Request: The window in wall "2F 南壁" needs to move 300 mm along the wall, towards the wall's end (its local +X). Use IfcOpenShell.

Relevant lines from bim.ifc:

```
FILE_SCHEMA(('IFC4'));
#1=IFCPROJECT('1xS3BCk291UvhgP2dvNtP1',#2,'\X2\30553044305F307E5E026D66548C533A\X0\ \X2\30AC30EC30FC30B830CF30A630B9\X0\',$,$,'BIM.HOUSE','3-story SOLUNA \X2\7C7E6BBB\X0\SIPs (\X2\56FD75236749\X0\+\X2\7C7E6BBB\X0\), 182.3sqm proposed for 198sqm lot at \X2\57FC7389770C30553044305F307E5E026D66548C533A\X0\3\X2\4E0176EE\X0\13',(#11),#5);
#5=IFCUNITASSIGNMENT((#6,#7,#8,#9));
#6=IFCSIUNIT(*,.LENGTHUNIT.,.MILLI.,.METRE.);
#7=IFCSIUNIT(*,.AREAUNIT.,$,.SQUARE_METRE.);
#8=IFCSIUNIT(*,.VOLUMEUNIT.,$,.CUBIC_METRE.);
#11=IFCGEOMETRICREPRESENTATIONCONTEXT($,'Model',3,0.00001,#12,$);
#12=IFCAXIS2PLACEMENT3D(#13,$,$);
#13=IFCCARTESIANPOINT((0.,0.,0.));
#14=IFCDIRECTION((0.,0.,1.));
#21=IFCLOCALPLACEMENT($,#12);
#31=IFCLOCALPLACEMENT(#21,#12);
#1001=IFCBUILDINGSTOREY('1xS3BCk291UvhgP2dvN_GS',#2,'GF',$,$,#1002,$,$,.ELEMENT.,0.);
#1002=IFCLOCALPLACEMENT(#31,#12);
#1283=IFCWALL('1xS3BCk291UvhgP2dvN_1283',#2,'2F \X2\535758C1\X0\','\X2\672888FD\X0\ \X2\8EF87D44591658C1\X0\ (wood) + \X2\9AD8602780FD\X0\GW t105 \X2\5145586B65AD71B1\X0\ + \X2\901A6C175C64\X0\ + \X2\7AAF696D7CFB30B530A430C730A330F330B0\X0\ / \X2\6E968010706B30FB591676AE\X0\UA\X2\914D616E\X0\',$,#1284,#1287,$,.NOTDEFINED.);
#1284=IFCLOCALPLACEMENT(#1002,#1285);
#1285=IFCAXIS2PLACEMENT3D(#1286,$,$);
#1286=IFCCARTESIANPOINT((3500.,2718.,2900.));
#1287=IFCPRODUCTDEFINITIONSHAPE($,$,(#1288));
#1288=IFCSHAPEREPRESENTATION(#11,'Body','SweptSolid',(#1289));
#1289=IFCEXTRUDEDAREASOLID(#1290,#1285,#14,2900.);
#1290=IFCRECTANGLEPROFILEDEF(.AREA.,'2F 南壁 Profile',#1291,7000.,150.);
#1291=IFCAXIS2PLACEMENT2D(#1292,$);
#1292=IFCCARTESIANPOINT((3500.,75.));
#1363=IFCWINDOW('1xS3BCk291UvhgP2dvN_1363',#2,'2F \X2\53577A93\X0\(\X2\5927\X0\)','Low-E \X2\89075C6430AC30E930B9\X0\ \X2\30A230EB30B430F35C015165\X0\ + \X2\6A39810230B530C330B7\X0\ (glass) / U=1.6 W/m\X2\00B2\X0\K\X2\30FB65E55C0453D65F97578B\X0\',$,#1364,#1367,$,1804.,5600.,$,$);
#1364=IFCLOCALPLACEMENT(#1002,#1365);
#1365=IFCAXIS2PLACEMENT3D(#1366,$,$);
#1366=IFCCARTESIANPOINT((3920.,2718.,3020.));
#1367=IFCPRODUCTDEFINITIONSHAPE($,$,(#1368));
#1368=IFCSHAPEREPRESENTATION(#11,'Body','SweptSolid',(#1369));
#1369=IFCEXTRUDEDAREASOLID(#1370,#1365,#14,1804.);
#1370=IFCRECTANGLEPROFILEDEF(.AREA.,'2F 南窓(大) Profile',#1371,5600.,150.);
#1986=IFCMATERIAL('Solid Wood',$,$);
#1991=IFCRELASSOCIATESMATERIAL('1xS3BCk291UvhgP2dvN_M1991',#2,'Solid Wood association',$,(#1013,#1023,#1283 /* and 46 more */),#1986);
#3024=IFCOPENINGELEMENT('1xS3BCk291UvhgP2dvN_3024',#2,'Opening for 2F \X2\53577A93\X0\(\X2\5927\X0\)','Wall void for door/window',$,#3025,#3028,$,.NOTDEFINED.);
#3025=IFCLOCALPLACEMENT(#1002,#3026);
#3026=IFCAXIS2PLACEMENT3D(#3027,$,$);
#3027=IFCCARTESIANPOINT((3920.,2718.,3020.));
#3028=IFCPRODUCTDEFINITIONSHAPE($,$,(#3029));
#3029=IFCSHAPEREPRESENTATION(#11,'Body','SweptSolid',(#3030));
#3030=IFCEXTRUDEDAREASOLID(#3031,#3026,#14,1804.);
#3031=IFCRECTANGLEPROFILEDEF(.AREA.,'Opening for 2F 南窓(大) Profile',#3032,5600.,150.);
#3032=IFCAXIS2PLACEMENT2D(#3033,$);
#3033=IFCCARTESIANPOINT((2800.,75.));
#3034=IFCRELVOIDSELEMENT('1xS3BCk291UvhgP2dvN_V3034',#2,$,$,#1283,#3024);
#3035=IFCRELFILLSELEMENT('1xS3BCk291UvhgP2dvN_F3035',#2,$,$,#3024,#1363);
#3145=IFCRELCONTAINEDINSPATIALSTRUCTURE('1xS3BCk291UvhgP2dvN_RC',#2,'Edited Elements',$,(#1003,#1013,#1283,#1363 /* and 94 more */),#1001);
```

```python
import ifcopenshell
import ifcopenshell.api.geometry
import ifcopenshell.util.placement

model = ifcopenshell.open("bim.ifc")

window = model.by_id(1363)
opening = window.FillsVoids[0].RelatingOpeningElement
wall = opening.VoidsElements[0].RelatingBuildingElement

wall_matrix = ifcopenshell.util.placement.get_local_placement(wall.ObjectPlacement)
shift = wall_matrix[:3, 0] * 300.0
before = ifcopenshell.util.placement.get_local_placement(window.ObjectPlacement)[:3, 3].copy()

# The window is not placed relative to its opening, so move both.
for product in (opening, window):
    matrix = ifcopenshell.util.placement.get_local_placement(product.ObjectPlacement)
    matrix[:3, 3] += shift
    ifcopenshell.api.geometry.edit_object_placement(model, product=product, matrix=matrix, is_si=False)

after = ifcopenshell.util.placement.get_local_placement(window.ObjectPlacement)[:3, 3]
print("window moved by", (after - before).round(3) + 0.0)

model.write("bim_rev.ifc")
```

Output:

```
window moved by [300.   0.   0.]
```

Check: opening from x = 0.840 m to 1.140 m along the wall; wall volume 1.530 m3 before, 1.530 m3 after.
